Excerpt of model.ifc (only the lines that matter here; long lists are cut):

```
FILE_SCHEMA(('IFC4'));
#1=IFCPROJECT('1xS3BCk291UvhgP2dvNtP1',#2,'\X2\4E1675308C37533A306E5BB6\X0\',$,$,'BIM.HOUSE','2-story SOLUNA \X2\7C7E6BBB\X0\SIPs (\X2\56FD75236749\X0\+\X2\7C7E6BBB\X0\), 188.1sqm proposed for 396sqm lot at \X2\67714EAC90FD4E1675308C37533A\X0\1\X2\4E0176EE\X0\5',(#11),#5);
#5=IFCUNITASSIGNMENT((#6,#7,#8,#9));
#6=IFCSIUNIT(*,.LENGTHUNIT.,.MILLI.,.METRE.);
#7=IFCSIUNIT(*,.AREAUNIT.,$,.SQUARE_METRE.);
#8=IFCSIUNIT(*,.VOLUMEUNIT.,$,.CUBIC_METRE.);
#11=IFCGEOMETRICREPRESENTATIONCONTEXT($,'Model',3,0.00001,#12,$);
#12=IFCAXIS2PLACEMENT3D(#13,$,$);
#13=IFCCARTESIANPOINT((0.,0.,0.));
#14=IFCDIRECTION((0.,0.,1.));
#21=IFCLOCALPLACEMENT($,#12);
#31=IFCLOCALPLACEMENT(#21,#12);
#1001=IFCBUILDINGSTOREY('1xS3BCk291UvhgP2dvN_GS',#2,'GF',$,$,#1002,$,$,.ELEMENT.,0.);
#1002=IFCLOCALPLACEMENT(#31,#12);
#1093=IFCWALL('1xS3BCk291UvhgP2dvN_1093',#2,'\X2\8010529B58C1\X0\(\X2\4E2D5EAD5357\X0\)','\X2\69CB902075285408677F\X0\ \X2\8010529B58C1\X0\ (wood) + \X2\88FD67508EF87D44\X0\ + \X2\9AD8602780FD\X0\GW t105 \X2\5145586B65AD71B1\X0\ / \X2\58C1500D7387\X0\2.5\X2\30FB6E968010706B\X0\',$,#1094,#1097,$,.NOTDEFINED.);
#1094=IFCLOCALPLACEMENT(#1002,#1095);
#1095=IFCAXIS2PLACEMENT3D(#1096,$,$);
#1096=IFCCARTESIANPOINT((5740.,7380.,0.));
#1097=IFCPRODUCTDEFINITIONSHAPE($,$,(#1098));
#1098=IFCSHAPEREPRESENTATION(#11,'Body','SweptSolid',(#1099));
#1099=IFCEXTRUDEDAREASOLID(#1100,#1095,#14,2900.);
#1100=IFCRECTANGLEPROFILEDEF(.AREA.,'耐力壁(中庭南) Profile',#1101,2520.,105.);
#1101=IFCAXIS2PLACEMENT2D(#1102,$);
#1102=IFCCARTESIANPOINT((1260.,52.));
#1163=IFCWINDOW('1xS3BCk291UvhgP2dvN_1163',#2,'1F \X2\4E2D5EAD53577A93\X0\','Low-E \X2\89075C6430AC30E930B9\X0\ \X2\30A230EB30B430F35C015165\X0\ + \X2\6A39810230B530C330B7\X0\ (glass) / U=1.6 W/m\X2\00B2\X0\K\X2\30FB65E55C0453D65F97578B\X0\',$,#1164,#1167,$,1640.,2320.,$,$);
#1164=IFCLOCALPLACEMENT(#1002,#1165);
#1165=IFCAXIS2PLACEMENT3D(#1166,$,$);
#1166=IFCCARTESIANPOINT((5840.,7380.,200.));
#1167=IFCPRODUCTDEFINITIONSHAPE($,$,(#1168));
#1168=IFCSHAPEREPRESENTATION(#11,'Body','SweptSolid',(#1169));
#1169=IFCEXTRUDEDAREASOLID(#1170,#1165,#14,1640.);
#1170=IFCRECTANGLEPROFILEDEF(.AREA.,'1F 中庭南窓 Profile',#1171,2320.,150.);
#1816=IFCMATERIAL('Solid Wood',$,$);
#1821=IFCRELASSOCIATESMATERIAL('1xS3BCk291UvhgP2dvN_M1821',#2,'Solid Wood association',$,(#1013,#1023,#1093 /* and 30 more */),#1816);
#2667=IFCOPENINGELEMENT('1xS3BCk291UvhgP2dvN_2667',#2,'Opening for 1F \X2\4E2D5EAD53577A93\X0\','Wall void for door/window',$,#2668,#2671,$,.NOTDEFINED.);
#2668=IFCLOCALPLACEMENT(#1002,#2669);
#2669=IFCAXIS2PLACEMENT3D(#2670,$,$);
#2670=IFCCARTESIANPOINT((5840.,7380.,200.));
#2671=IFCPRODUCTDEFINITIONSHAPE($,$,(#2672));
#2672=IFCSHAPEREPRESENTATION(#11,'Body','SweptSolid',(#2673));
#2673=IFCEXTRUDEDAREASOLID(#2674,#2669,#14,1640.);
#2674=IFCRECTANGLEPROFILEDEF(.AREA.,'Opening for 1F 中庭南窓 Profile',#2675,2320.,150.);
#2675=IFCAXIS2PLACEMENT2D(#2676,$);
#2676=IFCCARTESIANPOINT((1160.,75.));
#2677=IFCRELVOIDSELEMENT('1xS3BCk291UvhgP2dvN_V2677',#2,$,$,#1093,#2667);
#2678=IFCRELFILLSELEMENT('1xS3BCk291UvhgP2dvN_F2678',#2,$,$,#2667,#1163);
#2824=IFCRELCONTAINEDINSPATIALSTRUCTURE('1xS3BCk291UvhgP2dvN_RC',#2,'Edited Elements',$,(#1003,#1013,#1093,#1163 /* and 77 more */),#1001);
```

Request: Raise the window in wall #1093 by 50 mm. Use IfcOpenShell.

```python
import numpy as np
import ifcopenshell
import ifcopenshell.api.geometry
import ifcopenshell.util.placement
import ifcopenshell.util.unit

model = ifcopenshell.open("model.ifc")
unit_scale = ifcopenshell.util.unit.calculate_unit_scale(model)

window = model.by_guid("1xS3BCk291UvhgP2dvN_1163")
opening = window.FillsVoids[0].RelatingOpeningElement
dz = 0.05 / unit_scale

shift = np.array([0.0, 0.0, dz])
# The window is not placed relative to its opening, so move both.
for product in (opening, window):
    matrix = ifcopenshell.util.placement.get_local_placement(product.ObjectPlacement)
    matrix[:3, 3] += shift
    ifcopenshell.api.geometry.edit_object_placement(model, product=product, matrix=matrix, is_si=False)

print(f"moved by {dz * unit_scale:+.3f} m")

model.write("model-out.ifc")
```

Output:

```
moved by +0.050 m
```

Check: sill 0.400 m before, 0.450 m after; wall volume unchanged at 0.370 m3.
